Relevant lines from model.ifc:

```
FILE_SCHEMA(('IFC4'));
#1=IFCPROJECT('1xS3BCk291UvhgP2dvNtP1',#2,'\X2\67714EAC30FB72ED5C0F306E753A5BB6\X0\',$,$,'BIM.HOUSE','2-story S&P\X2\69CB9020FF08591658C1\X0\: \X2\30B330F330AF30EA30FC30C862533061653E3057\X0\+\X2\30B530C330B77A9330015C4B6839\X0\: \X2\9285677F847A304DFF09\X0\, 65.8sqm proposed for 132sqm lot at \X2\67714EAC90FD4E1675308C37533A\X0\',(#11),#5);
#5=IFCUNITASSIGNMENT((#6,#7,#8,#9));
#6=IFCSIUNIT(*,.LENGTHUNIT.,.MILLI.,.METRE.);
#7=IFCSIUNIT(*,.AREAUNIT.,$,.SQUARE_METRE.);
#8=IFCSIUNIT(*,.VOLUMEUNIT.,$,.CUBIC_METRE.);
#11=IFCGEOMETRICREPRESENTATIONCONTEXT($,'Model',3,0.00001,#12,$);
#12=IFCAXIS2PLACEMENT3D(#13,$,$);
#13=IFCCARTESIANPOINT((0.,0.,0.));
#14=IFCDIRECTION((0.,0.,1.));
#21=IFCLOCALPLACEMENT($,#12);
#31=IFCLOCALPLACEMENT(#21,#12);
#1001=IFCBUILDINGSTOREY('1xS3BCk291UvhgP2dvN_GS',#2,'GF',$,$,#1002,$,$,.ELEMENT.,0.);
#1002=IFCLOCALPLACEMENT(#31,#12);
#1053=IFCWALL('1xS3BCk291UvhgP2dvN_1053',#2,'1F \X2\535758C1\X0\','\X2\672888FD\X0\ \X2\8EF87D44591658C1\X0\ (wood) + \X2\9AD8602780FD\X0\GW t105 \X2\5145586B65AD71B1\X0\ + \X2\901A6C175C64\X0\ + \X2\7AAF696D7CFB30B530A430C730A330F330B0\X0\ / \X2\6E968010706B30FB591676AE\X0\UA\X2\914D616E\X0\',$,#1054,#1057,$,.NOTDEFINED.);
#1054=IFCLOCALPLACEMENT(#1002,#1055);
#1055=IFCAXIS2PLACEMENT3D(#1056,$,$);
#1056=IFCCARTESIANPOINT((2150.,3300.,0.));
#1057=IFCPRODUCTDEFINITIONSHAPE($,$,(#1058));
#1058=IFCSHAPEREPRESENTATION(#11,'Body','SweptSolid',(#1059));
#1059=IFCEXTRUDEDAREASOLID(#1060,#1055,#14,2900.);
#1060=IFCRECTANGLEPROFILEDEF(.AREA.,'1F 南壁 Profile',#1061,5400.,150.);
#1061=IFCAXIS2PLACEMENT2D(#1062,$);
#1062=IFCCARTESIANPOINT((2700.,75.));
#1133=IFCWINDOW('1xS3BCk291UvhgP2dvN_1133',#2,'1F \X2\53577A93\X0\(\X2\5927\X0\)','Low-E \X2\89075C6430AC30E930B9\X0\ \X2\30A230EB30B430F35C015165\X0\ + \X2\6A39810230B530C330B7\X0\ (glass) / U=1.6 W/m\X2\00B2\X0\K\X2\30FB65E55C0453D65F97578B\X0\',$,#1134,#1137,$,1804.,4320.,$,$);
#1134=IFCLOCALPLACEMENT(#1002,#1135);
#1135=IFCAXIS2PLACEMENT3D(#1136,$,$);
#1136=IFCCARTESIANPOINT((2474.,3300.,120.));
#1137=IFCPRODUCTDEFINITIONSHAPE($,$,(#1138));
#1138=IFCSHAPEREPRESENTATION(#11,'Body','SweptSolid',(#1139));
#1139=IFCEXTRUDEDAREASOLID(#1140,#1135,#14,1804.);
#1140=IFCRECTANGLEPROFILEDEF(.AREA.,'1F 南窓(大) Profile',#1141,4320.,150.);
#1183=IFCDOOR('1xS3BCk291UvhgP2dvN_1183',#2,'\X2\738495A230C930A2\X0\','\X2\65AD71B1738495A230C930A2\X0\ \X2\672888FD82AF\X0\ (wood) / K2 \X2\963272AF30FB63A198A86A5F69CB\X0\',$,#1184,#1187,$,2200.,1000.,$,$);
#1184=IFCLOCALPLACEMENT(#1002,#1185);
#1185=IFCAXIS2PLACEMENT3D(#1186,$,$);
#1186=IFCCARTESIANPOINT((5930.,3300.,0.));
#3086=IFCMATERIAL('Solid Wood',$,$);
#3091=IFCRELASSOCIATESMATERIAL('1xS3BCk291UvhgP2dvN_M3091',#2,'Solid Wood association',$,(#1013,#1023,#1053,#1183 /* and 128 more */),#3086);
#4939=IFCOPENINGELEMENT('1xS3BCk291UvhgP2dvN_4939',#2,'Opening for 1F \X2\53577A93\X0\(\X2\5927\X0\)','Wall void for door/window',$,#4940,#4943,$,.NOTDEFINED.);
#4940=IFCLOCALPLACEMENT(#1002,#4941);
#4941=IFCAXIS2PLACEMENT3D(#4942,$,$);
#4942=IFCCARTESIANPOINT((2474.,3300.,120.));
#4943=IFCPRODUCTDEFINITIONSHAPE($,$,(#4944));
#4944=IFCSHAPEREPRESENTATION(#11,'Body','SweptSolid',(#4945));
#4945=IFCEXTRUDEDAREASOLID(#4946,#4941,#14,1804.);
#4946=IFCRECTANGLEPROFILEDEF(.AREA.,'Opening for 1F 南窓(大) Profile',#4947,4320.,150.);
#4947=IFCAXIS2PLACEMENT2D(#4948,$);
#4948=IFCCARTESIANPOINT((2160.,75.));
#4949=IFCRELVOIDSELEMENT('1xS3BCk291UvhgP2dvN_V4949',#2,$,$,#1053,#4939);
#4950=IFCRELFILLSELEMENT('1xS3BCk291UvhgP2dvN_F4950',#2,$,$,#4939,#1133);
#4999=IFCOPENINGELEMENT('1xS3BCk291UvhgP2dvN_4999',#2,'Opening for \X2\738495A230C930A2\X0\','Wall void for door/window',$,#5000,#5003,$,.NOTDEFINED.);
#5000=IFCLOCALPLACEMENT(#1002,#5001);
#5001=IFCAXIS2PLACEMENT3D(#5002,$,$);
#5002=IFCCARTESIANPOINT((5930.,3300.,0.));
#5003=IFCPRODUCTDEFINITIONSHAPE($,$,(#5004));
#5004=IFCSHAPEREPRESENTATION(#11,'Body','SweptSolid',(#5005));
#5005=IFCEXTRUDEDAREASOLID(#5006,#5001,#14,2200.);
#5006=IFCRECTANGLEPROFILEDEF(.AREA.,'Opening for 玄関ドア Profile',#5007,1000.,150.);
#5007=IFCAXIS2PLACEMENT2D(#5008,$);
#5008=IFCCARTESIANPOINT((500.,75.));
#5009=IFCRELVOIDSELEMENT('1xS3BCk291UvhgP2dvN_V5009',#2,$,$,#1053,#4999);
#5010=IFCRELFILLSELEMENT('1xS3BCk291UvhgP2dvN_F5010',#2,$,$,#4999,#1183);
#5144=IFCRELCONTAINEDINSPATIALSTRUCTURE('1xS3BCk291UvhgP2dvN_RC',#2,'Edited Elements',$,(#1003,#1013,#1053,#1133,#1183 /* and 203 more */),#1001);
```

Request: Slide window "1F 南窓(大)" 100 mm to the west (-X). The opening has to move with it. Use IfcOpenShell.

```python
import ifcopenshell
import ifcopenshell.api.geometry
import ifcopenshell.util.placement
import ifcopenshell.util.unit

model = ifcopenshell.open("model.ifc")
unit_scale = ifcopenshell.util.unit.calculate_unit_scale(model)

window = model.by_guid("1xS3BCk291UvhgP2dvN_1133")
opening = window.FillsVoids[0].RelatingOpeningElement
wall = opening.VoidsElements[0].RelatingBuildingElement

wall_matrix = ifcopenshell.util.placement.get_local_placement(wall.ObjectPlacement)
shift = wall_matrix[:3, 0] * -0.1 / unit_scale
before = ifcopenshell.util.placement.get_local_placement(window.ObjectPlacement)[:3, 3].copy()

# The window is not placed relative to its opening, so move both.
for product in (opening, window):
    matrix = ifcopenshell.util.placement.get_local_placement(product.ObjectPlacement)
    matrix[:3, 3] += shift
    ifcopenshell.api.geometry.edit_object_placement(model, product=product, matrix=matrix, is_si=False)

after = ifcopenshell.util.placement.get_local_placement(window.ObjectPlacement)[:3, 3]
print("window moved by", (after - before).round(3) + 0.0)

model.write("model_rev.ifc")
```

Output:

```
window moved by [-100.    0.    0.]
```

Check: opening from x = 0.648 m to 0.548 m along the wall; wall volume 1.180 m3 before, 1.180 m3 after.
